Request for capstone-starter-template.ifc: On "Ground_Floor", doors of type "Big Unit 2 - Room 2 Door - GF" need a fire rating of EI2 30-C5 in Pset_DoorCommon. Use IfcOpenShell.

First a look at what the model holds.

```python
import ifcopenshell
import ifcopenshell.util.element

model = ifcopenshell.open("capstone-starter-template.ifc")
print(model.schema)
storey = next(s for s in model.by_type("IfcBuildingStorey") if s.Name == "Ground_Floor")
doors = [e for e in ifcopenshell.util.element.get_decomposition(storey) if e.is_a("IfcDoor")]
seen = {}
for e in doors:
    element_type = ifcopenshell.util.element.get_type(e)
    key = (element_type.Name if element_type != e and element_type else None, ifcopenshell.util.element.get_pset(e, "Pset_DoorCommon", "FireRating"))
    seen[key] = seen.get(key, 0) + 1
for (name, value), count in sorted(seen.items(), key=str):
    print(count, "x", name, "|", value)
```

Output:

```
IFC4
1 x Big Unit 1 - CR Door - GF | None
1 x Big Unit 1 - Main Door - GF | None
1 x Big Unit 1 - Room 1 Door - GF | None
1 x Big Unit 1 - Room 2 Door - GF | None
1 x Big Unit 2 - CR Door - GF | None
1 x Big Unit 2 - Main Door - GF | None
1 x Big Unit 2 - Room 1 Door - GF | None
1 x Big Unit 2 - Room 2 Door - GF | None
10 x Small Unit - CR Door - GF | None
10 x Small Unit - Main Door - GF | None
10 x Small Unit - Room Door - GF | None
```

```python
import ifcopenshell
import ifcopenshell.api.pset
import ifcopenshell.util.element

model = ifcopenshell.open("capstone-starter-template.ifc")

storey = next(s for s in model.by_type("IfcBuildingStorey") if s.Name == "Ground_Floor")
doors = [e for e in ifcopenshell.util.element.get_decomposition(storey) if e.is_a("IfcDoor")]

count = 0
for e in doors:
    element_type = ifcopenshell.util.element.get_type(e)
    if element_type in (None, e) or element_type.Name != "Big Unit 2 - Room 2 Door - GF":
        continue
    # add_pset returns the element's existing set when there is one.
    pset = ifcopenshell.api.pset.add_pset(model, product=e, name="Pset_DoorCommon")
    ifcopenshell.api.pset.edit_pset(model, pset=pset, properties={"FireRating": "EI2 30-C5"})
    count += 1

print(count, "doors updated")

model.write("capstone-starter-template_rev.ifc")
```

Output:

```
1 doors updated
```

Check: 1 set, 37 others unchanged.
